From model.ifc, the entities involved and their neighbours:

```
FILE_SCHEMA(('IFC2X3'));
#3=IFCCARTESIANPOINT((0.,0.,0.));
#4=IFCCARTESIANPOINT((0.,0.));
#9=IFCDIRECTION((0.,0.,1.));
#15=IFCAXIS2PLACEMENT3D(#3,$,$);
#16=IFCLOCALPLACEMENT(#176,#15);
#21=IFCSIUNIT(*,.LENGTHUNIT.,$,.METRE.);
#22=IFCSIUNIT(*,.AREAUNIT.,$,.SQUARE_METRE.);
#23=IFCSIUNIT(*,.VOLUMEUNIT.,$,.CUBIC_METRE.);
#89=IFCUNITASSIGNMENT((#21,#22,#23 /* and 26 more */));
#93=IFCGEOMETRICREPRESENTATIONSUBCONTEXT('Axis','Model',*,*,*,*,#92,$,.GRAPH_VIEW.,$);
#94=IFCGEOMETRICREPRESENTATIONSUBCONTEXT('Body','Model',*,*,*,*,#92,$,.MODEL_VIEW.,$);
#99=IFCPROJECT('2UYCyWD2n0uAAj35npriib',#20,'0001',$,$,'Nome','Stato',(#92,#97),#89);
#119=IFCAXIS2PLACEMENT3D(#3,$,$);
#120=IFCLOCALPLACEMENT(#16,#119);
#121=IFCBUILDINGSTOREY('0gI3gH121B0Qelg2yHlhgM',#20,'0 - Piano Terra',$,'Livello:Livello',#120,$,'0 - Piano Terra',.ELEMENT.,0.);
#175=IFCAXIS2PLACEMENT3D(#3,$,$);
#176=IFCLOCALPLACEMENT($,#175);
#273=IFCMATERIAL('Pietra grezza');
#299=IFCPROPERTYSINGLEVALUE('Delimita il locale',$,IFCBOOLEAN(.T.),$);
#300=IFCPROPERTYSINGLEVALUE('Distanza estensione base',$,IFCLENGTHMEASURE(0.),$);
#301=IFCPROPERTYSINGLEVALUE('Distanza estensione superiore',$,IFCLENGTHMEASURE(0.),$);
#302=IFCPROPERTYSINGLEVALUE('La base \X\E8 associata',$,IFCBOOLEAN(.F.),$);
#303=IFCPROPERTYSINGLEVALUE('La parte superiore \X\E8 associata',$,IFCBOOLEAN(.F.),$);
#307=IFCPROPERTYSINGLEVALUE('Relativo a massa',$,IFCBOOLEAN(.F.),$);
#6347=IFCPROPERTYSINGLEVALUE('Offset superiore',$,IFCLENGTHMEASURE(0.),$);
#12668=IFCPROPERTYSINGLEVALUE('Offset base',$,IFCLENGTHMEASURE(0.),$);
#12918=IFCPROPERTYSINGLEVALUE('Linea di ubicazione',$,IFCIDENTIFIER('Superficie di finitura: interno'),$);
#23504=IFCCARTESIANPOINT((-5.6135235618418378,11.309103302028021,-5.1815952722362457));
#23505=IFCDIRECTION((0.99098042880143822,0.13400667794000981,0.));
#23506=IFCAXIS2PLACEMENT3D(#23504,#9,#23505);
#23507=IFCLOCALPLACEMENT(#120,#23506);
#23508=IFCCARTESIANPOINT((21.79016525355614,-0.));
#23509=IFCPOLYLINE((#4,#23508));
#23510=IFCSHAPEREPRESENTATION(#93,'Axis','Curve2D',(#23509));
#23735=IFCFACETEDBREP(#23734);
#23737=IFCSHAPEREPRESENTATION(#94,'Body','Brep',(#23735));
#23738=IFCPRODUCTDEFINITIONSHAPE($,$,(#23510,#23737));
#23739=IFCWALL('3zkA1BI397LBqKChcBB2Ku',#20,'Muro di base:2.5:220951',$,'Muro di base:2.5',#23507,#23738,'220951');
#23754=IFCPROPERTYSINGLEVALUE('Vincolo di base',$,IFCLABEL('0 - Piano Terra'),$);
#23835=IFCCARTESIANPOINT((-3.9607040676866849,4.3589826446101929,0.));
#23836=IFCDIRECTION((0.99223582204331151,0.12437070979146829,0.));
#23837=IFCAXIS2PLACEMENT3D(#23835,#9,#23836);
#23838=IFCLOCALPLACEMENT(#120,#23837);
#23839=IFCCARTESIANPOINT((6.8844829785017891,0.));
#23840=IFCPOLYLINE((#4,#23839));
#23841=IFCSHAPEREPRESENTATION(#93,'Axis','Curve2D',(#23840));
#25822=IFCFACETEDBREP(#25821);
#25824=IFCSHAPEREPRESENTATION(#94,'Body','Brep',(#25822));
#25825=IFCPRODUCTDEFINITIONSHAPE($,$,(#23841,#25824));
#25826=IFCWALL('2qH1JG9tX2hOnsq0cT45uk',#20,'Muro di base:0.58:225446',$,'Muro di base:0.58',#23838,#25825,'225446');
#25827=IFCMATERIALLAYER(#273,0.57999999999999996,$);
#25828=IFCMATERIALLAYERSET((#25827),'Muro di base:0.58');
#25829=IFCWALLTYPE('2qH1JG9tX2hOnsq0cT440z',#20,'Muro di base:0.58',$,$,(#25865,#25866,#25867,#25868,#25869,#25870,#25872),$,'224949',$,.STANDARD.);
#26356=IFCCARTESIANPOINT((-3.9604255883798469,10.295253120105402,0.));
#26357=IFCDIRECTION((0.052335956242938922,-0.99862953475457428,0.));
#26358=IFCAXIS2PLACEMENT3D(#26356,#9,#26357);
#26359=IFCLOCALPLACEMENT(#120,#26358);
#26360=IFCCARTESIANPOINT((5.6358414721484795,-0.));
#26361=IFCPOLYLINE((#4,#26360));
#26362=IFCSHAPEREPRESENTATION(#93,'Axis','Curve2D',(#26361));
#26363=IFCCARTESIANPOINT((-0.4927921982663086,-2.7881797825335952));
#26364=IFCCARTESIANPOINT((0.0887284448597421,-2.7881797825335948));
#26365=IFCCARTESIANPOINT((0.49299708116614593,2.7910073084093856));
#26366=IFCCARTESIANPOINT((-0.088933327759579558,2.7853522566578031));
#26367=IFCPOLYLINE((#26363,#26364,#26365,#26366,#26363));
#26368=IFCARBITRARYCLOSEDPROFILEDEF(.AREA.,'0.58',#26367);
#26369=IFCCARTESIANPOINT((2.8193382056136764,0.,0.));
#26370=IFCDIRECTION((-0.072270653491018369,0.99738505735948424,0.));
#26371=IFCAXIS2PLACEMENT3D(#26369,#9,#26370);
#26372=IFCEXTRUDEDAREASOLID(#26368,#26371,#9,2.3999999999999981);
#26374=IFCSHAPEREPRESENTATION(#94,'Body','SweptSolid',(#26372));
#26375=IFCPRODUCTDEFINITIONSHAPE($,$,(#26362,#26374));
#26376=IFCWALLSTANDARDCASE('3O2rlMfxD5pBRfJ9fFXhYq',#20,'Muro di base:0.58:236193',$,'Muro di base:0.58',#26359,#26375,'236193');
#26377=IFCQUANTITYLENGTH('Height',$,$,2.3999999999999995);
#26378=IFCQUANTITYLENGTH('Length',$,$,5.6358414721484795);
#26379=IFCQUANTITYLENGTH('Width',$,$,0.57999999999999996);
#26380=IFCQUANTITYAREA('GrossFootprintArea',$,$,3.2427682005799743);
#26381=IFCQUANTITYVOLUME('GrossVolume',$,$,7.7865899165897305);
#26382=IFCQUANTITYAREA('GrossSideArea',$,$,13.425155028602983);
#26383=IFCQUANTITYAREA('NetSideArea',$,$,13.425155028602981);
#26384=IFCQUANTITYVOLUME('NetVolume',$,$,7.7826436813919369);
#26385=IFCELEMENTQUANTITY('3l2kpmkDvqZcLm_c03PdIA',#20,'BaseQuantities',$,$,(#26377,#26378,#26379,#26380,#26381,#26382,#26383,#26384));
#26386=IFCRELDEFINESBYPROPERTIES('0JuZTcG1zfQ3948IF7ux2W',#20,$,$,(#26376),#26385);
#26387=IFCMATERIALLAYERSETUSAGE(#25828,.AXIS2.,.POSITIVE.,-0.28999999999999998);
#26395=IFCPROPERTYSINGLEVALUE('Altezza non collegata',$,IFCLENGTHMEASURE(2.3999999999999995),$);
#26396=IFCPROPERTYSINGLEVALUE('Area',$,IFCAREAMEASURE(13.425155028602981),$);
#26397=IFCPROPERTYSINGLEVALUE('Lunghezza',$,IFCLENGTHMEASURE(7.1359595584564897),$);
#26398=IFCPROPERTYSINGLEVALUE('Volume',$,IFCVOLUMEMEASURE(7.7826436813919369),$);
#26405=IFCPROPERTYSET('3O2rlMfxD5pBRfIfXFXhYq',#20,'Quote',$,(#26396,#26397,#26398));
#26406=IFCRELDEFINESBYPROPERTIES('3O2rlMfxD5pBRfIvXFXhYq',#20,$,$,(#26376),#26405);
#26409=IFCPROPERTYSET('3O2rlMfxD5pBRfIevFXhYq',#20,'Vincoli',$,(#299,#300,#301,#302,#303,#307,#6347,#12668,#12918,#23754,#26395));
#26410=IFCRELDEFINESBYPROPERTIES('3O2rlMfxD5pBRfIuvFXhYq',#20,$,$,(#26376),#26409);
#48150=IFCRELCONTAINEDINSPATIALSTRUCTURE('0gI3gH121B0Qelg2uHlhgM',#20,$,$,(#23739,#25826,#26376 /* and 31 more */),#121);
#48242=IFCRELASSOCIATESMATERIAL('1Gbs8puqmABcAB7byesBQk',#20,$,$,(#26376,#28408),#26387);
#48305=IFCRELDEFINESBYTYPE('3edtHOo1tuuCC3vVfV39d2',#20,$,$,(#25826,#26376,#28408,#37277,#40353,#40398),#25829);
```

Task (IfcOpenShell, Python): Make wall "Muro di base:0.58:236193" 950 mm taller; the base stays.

```python
import ifcopenshell
import ifcopenshell.api.pset
import ifcopenshell.geom
import ifcopenshell.util.element
import ifcopenshell.util.representation
import ifcopenshell.util.shape
import ifcopenshell.util.unit

model = ifcopenshell.open("model.ifc")
unit_scale = ifcopenshell.util.unit.calculate_unit_scale(model)
area_scale = ifcopenshell.util.unit.calculate_unit_scale(model, "AREAUNIT")
volume_scale = ifcopenshell.util.unit.calculate_unit_scale(model, "VOLUMEUNIT")
settings = ifcopenshell.geom.settings()


def volume(element):
    """Net volume in cubic metres, openings subtracted."""
    shape = ifcopenshell.geom.create_shape(settings, element)
    return ifcopenshell.util.shape.get_volume(shape.geometry)


wall = model.by_guid("3O2rlMfxD5pBRfJ9fFXhYq")
before = volume(wall)

body = ifcopenshell.util.representation.get_representation(wall, "Model", "Body")
solid = body.Items[0]
old_height = solid.Depth
solid.Depth += 0.95
after = volume(wall)
thickness = 0.58  # wall thickness in metres

# Update the stored height, areas and volumes.
qto = model.by_id(ifcopenshell.util.element.get_pset(wall, "BaseQuantities", should_inherit=False)["id"])
ifcopenshell.api.pset.edit_qto(model, qto=qto, properties={
    "Height": solid.Depth,
    "GrossVolume": ifcopenshell.util.element.get_pset(wall, "BaseQuantities", "GrossVolume") * solid.Depth / old_height,
    "GrossSideArea": ifcopenshell.util.element.get_pset(wall, "BaseQuantities", "GrossSideArea") * solid.Depth / old_height,
    "NetSideArea": after / thickness / area_scale,
    "NetVolume": after / volume_scale,
})
pset = model.by_id(ifcopenshell.util.element.get_pset(wall, "Quote", should_inherit=False)["id"])
ifcopenshell.api.pset.edit_pset(model, pset=pset, properties={
    "Area": model.create_entity("IfcAreaMeasure", after / thickness / area_scale),
    "Volume": model.create_entity("IfcVolumeMeasure", after / volume_scale),
})
pset = model.by_id(ifcopenshell.util.element.get_pset(wall, "Vincoli", should_inherit=False)["id"])
ifcopenshell.api.pset.edit_pset(model, pset=pset, properties={
    "Altezza non collegata": model.create_entity("IfcLengthMeasure", solid.Depth),
})

print(f"height {old_height:g} -> {solid.Depth:g}, volume {before:.3f} -> {after:.3f} m3")

model.write("model_v2.ifc")
```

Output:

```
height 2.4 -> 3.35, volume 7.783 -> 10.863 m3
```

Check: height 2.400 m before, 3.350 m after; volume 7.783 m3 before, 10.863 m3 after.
